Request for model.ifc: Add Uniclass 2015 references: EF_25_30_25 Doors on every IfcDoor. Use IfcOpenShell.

First a look at what the model holds.

```python
import ifcopenshell

model = ifcopenshell.open("model.ifc")
print(model.schema)
print("classifications:", [c.Name for c in model.by_type("IfcClassification")])
for ifc_class in ("IfcDoor", "IfcRoof", "IfcStair", "IfcWall", "IfcWindow"):
    print(ifc_class, len(model.by_type(ifc_class)))
```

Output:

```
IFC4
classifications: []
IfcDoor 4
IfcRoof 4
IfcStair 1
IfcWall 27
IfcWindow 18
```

```python
import ifcopenshell
import ifcopenshell.api.classification

model = ifcopenshell.open("model.ifc")

system = ifcopenshell.api.classification.add_classification(model, classification="Uniclass 2015")

codes = {
    "IfcDoor": ("EF_25_30_25", "Doors"),
}
for ifc_class, (code, name) in codes.items():
    products = model.by_type(ifc_class)
    ifcopenshell.api.classification.add_reference(
        model, products=products, classification=system, identification=code, name=name
    )
    print(code, len(products))

model.write("model_rev.ifc")
```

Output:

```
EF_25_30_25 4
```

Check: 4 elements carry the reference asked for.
